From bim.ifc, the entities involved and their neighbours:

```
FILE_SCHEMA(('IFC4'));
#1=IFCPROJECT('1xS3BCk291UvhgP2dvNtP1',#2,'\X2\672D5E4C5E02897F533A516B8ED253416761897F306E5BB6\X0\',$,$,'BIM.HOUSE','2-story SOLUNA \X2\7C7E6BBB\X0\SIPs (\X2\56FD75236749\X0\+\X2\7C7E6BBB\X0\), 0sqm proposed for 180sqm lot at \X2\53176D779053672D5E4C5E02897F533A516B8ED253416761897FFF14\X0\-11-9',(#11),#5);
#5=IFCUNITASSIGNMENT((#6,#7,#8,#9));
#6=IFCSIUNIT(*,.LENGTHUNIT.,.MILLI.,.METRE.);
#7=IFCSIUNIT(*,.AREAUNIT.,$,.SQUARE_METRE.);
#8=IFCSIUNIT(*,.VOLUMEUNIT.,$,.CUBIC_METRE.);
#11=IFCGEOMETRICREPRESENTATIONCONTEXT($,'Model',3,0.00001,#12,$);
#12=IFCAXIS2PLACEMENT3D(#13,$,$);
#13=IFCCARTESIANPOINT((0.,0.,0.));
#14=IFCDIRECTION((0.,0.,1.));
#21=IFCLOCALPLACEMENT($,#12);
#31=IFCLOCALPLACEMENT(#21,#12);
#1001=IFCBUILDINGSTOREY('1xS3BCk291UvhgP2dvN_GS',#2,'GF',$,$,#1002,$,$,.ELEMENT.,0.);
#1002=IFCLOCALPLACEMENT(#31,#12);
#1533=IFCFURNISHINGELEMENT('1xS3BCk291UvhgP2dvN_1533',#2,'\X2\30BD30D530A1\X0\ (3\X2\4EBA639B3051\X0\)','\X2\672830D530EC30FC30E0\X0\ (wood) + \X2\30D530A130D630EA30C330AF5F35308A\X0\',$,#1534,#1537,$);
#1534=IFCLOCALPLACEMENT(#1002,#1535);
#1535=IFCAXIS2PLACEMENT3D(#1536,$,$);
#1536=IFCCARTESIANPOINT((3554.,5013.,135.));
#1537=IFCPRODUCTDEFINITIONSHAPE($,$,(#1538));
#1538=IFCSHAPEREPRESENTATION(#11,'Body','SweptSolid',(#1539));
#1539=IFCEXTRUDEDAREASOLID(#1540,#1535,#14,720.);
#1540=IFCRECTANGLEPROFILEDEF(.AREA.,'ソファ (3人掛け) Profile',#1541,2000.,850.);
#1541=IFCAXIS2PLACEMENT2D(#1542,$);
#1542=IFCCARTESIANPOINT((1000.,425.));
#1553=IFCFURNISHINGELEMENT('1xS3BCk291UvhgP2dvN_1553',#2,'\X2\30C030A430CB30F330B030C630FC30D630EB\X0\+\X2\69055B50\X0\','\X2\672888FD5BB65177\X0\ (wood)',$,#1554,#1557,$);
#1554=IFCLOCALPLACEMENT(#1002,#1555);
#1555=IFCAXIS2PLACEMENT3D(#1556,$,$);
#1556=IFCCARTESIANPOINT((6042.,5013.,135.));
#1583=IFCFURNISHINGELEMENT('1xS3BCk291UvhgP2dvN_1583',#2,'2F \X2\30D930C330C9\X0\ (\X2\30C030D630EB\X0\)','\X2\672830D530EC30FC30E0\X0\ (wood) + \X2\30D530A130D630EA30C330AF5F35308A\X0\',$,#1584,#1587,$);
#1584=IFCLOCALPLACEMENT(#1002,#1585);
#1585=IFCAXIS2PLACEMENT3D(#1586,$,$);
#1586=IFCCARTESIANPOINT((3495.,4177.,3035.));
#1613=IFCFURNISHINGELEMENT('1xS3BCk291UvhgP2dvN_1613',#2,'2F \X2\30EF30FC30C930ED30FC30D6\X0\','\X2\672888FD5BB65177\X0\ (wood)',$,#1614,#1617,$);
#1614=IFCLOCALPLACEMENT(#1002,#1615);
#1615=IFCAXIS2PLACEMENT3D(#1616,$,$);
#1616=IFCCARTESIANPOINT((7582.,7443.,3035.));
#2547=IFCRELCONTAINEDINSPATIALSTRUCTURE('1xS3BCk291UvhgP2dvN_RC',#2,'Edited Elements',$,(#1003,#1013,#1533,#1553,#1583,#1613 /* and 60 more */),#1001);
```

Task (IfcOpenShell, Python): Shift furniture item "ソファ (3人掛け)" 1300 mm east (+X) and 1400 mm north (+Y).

```python
import ifcopenshell
import ifcopenshell.api.geometry
import ifcopenshell.util.placement
import ifcopenshell.util.unit

model = ifcopenshell.open("bim.ifc")
unit_scale = ifcopenshell.util.unit.calculate_unit_scale(model)

item = model.by_guid("1xS3BCk291UvhgP2dvN_1533")
matrix = ifcopenshell.util.placement.get_local_placement(item.ObjectPlacement)
matrix[0, 3] += 1.3 / unit_scale
matrix[1, 3] += 1.4 / unit_scale
ifcopenshell.api.geometry.edit_object_placement(model, product=item, matrix=matrix, is_si=False)

print(ifcopenshell.util.placement.get_local_placement(item.ObjectPlacement).round(3) + 0.0)

model.write("bim_edited.ifc")
```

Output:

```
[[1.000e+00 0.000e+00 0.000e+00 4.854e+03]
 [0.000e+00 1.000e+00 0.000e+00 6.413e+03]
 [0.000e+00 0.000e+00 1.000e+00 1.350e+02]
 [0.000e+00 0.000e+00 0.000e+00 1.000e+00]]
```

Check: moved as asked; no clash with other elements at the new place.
